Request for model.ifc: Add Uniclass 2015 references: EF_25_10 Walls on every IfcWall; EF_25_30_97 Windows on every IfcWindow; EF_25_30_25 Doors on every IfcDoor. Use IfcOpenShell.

First a look at what the model holds.

```python
import ifcopenshell

model = ifcopenshell.open("model.ifc")
print(model.schema)
print("classifications:", [c.Name for c in model.by_type("IfcClassification")])
for ifc_class in ("IfcDoor", "IfcRoof", "IfcStair", "IfcWall", "IfcWindow"):
    print(ifc_class, len(model.by_type(ifc_class)))
```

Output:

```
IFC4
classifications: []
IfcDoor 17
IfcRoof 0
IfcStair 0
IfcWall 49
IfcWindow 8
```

```python
import ifcopenshell
import ifcopenshell.api.classification

model = ifcopenshell.open("model.ifc")

system = ifcopenshell.api.classification.add_classification(model, classification="Uniclass 2015")

codes = {
    "IfcWall": ("EF_25_10", "Walls"),
    "IfcWindow": ("EF_25_30_97", "Windows"),
    "IfcDoor": ("EF_25_30_25", "Doors"),
}
for ifc_class, (code, name) in codes.items():
    products = model.by_type(ifc_class)
    ifcopenshell.api.classification.add_reference(
        model, products=products, classification=system, identification=code, name=name
    )
    print(code, len(products))

model.write("model_updated.ifc")
```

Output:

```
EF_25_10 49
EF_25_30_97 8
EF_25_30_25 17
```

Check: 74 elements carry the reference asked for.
